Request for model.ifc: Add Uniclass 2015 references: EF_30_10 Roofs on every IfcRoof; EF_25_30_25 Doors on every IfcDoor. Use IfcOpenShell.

First a look at what the model holds.

```python
import ifcopenshell

model = ifcopenshell.open("model.ifc")
print(model.schema)
print("classifications:", [c.Name for c in model.by_type("IfcClassification")])
for ifc_class in ("IfcDoor", "IfcRoof", "IfcStair", "IfcWall", "IfcWindow"):
    print(ifc_class, len(model.by_type(ifc_class)))
```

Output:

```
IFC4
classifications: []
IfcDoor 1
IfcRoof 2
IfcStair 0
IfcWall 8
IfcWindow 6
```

```python
import ifcopenshell
import ifcopenshell.api.classification

model = ifcopenshell.open("model.ifc")

system = ifcopenshell.api.classification.add_classification(model, classification="Uniclass 2015")

codes = {
    "IfcRoof": ("EF_30_10", "Roofs"),
    "IfcDoor": ("EF_25_30_25", "Doors"),
}
for ifc_class, (code, name) in codes.items():
    products = model.by_type(ifc_class)
    ifcopenshell.api.classification.add_reference(
        model, products=products, classification=system, identification=code, name=name
    )
    print(code, len(products))

model.write("model_rev.ifc")
```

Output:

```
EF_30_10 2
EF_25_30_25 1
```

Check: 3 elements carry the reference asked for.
